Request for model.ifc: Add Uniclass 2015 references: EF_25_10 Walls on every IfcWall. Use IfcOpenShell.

First a look at what the model holds.

```python
import ifcopenshell

model = ifcopenshell.open("model.ifc")
print(model.schema)
print("classifications:", [c.Name for c in model.by_type("IfcClassification")])
for ifc_class in ("IfcDoor", "IfcRoof", "IfcStair", "IfcWall", "IfcWindow"):
    print(ifc_class, len(model.by_type(ifc_class)))
```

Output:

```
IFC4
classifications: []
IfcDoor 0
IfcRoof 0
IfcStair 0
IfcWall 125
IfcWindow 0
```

```python
import ifcopenshell
import ifcopenshell.api.classification

model = ifcopenshell.open("model.ifc")

system = ifcopenshell.api.classification.add_classification(model, classification="Uniclass 2015")

codes = {
    "IfcWall": ("EF_25_10", "Walls"),
}
for ifc_class, (code, name) in codes.items():
    products = model.by_type(ifc_class)
    ifcopenshell.api.classification.add_reference(
        model, products=products, classification=system, identification=code, name=name
    )
    print(code, len(products))

model.write("model-out.ifc")
```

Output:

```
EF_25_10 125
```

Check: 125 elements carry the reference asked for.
